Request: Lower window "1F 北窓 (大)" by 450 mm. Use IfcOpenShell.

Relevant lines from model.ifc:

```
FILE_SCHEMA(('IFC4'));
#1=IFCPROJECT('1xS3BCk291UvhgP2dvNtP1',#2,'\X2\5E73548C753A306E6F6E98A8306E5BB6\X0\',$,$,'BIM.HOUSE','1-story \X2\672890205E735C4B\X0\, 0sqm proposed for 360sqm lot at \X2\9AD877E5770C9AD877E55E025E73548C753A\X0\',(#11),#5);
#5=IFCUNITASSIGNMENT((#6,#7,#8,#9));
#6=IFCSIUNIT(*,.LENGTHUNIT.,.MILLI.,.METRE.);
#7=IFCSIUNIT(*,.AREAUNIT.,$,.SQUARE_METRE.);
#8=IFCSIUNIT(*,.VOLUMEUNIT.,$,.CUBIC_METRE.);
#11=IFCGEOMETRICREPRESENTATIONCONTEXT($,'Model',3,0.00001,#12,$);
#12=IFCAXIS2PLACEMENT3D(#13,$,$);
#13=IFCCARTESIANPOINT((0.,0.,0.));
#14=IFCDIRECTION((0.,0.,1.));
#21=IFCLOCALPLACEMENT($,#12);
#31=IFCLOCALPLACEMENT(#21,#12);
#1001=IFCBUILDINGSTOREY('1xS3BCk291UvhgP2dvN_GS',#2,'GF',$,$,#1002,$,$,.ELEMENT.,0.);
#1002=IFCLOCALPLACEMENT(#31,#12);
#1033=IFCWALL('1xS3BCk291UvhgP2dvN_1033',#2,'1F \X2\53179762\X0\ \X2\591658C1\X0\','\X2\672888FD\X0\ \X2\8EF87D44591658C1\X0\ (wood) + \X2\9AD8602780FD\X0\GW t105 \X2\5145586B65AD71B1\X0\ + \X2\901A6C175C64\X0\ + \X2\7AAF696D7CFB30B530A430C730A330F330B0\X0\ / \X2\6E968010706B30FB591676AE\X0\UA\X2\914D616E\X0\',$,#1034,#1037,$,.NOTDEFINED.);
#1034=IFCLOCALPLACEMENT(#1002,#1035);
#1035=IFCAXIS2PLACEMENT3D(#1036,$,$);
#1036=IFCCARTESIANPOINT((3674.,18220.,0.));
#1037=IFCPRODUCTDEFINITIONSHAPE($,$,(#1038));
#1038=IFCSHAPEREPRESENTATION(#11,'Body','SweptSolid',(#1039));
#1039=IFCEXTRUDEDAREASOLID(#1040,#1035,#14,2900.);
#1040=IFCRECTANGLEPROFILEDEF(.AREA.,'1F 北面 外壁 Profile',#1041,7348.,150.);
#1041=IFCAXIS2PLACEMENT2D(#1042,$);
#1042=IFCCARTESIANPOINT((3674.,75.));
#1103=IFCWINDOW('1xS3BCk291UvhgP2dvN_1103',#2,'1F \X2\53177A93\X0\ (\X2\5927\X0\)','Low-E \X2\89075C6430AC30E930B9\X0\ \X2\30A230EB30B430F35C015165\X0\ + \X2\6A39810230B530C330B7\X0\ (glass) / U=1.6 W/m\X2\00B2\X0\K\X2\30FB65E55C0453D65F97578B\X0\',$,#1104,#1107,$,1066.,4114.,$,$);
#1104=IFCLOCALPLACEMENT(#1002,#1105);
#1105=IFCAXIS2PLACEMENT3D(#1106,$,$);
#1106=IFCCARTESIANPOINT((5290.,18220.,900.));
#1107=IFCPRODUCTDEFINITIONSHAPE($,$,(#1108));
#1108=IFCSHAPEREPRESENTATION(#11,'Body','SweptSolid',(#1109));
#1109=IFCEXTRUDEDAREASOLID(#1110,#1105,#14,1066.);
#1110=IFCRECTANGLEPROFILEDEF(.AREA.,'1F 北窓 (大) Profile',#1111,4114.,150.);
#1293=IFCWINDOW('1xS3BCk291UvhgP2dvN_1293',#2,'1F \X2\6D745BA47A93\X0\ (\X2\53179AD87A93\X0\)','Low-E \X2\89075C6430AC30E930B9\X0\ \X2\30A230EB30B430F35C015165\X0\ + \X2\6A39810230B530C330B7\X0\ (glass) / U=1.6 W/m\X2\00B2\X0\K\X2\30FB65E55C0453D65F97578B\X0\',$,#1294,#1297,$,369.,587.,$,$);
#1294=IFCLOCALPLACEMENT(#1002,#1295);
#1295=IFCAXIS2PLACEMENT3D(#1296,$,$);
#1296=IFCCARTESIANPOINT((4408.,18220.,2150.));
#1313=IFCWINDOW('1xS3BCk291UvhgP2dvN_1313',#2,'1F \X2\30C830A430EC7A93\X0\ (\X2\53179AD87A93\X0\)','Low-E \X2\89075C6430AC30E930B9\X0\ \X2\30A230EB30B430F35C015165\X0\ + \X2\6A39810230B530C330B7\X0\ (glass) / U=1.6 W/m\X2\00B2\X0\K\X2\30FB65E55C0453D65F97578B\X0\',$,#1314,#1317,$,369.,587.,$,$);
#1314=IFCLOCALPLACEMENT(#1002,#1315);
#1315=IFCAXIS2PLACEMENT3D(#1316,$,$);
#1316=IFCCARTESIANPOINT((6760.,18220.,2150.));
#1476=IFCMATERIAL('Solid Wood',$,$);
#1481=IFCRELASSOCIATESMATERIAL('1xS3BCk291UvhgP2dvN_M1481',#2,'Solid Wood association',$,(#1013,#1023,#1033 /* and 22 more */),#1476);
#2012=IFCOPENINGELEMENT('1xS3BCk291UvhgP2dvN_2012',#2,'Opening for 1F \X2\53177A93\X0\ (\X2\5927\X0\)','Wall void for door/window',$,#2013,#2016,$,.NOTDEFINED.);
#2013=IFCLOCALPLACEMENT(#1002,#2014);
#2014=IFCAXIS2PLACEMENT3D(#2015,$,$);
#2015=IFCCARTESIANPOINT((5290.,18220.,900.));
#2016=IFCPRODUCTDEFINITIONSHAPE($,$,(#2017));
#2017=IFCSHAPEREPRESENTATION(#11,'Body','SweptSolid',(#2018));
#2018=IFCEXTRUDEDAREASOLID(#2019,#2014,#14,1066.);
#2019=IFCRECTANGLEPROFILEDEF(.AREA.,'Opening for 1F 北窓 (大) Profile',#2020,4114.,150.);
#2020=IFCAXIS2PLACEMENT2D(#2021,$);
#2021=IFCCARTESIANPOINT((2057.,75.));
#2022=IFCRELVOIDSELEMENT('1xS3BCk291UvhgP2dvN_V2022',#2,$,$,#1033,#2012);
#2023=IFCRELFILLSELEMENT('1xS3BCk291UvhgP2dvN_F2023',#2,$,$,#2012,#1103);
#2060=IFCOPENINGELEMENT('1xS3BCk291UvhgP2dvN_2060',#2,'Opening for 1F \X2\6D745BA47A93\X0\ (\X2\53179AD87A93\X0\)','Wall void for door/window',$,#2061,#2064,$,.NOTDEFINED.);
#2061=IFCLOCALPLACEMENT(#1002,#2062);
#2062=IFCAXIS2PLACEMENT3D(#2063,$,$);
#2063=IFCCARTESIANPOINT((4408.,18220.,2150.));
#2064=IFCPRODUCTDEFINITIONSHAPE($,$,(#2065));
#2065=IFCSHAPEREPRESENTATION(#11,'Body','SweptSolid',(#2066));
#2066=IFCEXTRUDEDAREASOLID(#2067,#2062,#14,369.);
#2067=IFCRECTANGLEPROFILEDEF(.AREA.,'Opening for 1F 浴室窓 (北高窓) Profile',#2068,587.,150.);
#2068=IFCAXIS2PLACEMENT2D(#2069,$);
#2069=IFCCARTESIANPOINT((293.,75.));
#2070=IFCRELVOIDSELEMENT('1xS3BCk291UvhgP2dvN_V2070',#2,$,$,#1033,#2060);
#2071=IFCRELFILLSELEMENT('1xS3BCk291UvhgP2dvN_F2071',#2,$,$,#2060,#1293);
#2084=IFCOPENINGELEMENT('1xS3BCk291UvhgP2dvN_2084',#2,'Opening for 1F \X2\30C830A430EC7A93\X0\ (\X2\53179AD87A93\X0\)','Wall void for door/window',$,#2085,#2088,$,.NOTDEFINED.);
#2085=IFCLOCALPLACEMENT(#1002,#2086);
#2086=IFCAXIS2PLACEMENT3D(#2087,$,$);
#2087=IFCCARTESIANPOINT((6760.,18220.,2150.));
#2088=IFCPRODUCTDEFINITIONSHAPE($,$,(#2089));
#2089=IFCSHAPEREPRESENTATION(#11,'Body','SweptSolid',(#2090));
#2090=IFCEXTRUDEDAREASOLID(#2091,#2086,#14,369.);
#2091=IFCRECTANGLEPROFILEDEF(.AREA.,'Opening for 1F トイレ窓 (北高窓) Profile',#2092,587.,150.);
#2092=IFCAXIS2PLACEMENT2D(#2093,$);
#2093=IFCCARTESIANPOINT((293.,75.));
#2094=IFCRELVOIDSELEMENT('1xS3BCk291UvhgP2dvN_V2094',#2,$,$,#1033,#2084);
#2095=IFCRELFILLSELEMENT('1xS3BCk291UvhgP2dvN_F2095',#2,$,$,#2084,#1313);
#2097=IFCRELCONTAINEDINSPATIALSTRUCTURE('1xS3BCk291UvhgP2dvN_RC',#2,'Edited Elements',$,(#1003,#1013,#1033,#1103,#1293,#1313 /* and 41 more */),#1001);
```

```python
import numpy as np
import ifcopenshell
import ifcopenshell.api.geometry
import ifcopenshell.util.placement
import ifcopenshell.util.unit

model = ifcopenshell.open("model.ifc")
unit_scale = ifcopenshell.util.unit.calculate_unit_scale(model)

window = model.by_guid("1xS3BCk291UvhgP2dvN_1103")
opening = window.FillsVoids[0].RelatingOpeningElement
dz = -0.45 / unit_scale

shift = np.array([0.0, 0.0, dz])
# The window is not placed relative to its opening, so move both.
for product in (opening, window):
    matrix = ifcopenshell.util.placement.get_local_placement(product.ObjectPlacement)
    matrix[:3, 3] += shift
    ifcopenshell.api.geometry.edit_object_placement(model, product=product, matrix=matrix, is_si=False)

print(f"moved by {dz * unit_scale:+.3f} m")

model.write("model_rev.ifc")
```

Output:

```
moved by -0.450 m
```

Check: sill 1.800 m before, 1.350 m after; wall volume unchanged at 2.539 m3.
